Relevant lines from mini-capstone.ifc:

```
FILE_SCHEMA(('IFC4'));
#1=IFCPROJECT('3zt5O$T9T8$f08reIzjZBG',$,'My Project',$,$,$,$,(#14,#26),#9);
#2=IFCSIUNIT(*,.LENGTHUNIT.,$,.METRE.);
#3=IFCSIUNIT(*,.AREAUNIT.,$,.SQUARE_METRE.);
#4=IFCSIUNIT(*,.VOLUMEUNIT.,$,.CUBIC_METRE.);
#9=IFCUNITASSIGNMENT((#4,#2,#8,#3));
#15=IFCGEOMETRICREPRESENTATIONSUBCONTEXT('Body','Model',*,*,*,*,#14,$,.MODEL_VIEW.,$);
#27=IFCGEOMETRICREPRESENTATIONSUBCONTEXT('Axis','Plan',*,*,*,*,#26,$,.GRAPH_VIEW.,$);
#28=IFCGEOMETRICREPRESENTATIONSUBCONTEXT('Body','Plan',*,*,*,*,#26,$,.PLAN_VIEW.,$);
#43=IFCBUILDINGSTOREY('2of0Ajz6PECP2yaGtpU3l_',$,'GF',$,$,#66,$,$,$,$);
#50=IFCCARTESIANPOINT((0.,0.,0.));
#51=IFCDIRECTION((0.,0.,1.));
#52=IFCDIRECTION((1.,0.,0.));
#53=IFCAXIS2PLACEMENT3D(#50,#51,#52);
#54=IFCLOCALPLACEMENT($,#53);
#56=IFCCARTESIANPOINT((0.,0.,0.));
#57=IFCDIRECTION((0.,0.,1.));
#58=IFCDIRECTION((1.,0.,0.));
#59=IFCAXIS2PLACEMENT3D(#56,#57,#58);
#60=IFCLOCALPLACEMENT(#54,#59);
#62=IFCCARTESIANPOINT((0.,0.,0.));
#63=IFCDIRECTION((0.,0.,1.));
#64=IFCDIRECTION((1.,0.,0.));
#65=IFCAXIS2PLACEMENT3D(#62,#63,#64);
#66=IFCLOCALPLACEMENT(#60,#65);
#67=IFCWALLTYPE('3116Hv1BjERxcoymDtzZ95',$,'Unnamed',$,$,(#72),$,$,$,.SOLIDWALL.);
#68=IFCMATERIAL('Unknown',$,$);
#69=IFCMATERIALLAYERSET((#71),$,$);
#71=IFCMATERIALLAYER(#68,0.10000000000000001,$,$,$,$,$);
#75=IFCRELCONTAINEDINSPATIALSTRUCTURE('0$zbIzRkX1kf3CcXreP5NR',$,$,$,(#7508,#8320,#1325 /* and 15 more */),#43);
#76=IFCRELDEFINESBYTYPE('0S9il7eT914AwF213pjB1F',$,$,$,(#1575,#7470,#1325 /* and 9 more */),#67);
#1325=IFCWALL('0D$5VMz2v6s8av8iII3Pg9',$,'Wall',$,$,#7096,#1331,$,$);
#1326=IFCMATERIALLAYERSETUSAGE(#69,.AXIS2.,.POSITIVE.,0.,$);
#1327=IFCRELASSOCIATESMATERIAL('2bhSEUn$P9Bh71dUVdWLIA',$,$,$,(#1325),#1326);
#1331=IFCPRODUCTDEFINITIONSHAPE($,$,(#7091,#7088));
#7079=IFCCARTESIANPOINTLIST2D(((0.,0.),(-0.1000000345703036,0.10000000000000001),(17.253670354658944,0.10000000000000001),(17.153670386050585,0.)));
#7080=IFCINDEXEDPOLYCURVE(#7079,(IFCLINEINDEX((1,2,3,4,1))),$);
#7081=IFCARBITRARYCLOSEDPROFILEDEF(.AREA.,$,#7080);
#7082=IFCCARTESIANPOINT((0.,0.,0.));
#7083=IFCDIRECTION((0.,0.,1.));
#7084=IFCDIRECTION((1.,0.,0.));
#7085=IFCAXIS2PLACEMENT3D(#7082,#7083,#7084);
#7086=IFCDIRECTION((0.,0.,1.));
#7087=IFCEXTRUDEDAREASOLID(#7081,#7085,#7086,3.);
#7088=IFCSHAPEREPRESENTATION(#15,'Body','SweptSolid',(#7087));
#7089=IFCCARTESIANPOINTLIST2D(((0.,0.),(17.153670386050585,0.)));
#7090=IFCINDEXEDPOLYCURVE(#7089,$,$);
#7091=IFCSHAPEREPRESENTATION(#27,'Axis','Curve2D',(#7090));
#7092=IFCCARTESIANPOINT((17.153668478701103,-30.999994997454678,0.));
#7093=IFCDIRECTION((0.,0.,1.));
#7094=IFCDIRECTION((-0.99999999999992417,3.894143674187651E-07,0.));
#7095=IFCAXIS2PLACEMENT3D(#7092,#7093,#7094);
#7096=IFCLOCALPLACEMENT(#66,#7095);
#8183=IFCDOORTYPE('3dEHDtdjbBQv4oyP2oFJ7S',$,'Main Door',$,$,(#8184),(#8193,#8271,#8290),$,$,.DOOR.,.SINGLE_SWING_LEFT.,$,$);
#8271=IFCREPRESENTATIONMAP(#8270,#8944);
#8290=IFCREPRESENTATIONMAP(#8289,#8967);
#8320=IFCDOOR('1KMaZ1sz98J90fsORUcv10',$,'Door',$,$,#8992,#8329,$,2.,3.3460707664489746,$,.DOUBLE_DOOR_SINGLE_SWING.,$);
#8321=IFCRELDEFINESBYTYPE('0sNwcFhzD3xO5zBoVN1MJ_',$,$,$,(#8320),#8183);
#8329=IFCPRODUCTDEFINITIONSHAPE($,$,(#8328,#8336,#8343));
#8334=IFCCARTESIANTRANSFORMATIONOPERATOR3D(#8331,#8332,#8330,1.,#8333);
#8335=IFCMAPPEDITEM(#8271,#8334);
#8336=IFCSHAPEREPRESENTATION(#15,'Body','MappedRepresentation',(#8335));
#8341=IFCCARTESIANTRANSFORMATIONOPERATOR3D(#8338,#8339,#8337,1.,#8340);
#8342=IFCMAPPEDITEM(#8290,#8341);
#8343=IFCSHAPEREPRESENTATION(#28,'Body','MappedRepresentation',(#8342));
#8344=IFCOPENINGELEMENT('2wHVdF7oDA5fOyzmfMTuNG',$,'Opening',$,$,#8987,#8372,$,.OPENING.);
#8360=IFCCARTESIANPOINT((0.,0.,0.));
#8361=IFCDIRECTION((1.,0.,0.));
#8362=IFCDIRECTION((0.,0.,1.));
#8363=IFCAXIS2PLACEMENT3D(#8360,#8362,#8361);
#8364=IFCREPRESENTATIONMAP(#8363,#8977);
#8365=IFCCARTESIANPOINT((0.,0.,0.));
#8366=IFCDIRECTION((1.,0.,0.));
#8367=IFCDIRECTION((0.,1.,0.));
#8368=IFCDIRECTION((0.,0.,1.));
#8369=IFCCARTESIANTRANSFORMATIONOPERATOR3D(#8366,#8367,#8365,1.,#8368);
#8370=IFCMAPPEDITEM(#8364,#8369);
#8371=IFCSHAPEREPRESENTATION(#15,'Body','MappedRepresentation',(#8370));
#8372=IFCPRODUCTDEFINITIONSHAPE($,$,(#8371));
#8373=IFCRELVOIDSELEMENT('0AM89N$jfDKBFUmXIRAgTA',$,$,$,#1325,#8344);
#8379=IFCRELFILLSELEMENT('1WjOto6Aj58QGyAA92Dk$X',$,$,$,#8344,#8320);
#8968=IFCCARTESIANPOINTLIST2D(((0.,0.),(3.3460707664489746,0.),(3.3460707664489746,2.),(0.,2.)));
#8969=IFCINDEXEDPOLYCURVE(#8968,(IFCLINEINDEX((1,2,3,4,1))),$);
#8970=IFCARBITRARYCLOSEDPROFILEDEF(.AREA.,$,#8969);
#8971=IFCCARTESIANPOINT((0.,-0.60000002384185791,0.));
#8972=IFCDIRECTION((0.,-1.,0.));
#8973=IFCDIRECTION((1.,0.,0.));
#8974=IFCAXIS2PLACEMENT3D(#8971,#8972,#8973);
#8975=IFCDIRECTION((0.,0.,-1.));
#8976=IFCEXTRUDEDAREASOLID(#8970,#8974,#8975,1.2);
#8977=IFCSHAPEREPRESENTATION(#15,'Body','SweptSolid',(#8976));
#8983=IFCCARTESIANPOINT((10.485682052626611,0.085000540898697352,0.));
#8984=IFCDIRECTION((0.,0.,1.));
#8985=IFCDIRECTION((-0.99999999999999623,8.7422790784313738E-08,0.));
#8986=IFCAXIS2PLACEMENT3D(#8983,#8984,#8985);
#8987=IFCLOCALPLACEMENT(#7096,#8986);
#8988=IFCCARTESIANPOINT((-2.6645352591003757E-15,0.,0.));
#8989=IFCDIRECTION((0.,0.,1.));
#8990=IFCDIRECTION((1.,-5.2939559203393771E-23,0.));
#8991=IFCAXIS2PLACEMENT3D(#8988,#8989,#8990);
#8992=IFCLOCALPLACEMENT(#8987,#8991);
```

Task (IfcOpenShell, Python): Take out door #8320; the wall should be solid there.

```python
import ifcopenshell
import ifcopenshell.api.feature
import ifcopenshell.api.root
import ifcopenshell.geom
import ifcopenshell.util.shape

model = ifcopenshell.open("mini-capstone.ifc")
settings = ifcopenshell.geom.settings()


def volume(element):
    """Net volume in cubic metres, openings subtracted."""
    shape = ifcopenshell.geom.create_shape(settings, element)
    return ifcopenshell.util.shape.get_volume(shape.geometry)


door = model.by_id(8320)
opening = door.FillsVoids[0].RelatingOpeningElement
wall = opening.VoidsElements[0].RelatingBuildingElement
before = volume(wall)

ifcopenshell.api.root.remove_product(model, product=door)
ifcopenshell.api.feature.remove_feature(model, feature=opening)

after = volume(wall)

print(f"wall volume {before:.3f} -> {after:.3f} m3")

model.write("mini-capstone_rev.ifc")
```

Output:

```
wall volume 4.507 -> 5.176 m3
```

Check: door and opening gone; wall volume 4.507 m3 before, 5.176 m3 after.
